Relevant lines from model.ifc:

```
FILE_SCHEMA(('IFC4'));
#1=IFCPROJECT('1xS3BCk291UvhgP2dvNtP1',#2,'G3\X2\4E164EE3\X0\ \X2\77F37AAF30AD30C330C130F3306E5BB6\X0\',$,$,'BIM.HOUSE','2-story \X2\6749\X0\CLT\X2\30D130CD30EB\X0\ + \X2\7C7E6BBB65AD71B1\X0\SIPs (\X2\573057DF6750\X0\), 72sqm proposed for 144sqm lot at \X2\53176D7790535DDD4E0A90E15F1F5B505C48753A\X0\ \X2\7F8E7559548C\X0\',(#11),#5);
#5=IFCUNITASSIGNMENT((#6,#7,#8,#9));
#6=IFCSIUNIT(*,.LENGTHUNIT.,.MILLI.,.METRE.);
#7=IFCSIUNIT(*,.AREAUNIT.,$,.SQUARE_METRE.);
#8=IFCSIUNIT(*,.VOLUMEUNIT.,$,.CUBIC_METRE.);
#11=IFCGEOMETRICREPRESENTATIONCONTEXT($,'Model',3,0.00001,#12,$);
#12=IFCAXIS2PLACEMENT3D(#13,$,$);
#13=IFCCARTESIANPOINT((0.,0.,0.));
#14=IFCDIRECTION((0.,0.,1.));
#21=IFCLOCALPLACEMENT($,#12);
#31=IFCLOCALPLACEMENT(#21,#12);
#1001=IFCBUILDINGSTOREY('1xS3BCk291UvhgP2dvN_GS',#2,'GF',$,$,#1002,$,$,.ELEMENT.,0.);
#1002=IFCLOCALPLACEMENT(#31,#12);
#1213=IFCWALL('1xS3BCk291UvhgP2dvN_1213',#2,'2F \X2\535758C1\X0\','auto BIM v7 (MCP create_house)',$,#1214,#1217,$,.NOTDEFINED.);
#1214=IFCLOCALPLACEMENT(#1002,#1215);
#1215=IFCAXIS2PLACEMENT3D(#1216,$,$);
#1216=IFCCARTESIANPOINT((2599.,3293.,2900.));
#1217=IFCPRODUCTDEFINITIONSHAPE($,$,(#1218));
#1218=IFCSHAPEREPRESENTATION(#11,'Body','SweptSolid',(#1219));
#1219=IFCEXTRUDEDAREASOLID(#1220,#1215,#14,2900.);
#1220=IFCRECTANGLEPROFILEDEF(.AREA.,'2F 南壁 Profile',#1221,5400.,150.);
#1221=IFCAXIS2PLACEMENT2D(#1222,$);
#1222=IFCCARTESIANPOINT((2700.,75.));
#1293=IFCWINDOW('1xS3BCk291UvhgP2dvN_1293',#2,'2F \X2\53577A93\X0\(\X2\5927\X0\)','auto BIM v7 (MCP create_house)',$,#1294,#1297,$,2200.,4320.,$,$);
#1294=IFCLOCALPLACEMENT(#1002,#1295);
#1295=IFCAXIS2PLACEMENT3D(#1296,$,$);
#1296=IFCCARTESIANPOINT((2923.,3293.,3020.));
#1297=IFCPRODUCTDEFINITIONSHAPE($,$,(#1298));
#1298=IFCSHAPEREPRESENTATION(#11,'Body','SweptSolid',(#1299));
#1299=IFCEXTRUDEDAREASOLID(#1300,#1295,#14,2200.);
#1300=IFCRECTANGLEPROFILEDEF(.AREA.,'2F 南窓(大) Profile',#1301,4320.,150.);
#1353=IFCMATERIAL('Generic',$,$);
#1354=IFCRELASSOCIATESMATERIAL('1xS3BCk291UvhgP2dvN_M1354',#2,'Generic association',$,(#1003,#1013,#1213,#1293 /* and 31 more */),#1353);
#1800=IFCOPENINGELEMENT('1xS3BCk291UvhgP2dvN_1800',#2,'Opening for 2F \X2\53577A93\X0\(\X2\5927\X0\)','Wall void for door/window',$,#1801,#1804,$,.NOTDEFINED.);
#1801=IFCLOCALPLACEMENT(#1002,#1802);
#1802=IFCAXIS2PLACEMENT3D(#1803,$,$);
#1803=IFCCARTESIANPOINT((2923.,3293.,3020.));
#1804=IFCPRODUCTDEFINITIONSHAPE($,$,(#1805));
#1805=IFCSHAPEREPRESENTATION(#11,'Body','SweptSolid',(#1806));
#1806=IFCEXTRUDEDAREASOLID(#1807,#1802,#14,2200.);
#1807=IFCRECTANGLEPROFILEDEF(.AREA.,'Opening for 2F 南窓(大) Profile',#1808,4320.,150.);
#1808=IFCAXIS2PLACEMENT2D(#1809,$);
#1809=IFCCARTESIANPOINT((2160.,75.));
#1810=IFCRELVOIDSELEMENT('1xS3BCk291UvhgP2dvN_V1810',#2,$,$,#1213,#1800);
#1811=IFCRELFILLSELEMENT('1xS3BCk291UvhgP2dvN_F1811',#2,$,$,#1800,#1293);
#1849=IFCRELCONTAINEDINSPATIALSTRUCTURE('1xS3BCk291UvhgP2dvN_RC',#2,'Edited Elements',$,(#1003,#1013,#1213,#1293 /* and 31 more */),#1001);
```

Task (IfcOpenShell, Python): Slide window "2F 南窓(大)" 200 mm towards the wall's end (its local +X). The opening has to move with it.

```python
import ifcopenshell
import ifcopenshell.api.geometry
import ifcopenshell.util.placement

model = ifcopenshell.open("model.ifc")

window = model.by_guid("1xS3BCk291UvhgP2dvN_1293")
opening = window.FillsVoids[0].RelatingOpeningElement
wall = opening.VoidsElements[0].RelatingBuildingElement

wall_matrix = ifcopenshell.util.placement.get_local_placement(wall.ObjectPlacement)
shift = wall_matrix[:3, 0] * 200.0
before = ifcopenshell.util.placement.get_local_placement(window.ObjectPlacement)[:3, 3].copy()

# The window is not placed relative to its opening, so move both.
for product in (opening, window):
    matrix = ifcopenshell.util.placement.get_local_placement(product.ObjectPlacement)
    matrix[:3, 3] += shift
    ifcopenshell.api.geometry.edit_object_placement(model, product=product, matrix=matrix, is_si=False)

after = ifcopenshell.util.placement.get_local_placement(window.ObjectPlacement)[:3, 3]
print("window moved by", (after - before).round(3) + 0.0)

model.write("model_rev.ifc")
```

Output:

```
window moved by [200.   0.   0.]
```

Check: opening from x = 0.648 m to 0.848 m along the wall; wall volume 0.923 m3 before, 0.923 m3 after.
